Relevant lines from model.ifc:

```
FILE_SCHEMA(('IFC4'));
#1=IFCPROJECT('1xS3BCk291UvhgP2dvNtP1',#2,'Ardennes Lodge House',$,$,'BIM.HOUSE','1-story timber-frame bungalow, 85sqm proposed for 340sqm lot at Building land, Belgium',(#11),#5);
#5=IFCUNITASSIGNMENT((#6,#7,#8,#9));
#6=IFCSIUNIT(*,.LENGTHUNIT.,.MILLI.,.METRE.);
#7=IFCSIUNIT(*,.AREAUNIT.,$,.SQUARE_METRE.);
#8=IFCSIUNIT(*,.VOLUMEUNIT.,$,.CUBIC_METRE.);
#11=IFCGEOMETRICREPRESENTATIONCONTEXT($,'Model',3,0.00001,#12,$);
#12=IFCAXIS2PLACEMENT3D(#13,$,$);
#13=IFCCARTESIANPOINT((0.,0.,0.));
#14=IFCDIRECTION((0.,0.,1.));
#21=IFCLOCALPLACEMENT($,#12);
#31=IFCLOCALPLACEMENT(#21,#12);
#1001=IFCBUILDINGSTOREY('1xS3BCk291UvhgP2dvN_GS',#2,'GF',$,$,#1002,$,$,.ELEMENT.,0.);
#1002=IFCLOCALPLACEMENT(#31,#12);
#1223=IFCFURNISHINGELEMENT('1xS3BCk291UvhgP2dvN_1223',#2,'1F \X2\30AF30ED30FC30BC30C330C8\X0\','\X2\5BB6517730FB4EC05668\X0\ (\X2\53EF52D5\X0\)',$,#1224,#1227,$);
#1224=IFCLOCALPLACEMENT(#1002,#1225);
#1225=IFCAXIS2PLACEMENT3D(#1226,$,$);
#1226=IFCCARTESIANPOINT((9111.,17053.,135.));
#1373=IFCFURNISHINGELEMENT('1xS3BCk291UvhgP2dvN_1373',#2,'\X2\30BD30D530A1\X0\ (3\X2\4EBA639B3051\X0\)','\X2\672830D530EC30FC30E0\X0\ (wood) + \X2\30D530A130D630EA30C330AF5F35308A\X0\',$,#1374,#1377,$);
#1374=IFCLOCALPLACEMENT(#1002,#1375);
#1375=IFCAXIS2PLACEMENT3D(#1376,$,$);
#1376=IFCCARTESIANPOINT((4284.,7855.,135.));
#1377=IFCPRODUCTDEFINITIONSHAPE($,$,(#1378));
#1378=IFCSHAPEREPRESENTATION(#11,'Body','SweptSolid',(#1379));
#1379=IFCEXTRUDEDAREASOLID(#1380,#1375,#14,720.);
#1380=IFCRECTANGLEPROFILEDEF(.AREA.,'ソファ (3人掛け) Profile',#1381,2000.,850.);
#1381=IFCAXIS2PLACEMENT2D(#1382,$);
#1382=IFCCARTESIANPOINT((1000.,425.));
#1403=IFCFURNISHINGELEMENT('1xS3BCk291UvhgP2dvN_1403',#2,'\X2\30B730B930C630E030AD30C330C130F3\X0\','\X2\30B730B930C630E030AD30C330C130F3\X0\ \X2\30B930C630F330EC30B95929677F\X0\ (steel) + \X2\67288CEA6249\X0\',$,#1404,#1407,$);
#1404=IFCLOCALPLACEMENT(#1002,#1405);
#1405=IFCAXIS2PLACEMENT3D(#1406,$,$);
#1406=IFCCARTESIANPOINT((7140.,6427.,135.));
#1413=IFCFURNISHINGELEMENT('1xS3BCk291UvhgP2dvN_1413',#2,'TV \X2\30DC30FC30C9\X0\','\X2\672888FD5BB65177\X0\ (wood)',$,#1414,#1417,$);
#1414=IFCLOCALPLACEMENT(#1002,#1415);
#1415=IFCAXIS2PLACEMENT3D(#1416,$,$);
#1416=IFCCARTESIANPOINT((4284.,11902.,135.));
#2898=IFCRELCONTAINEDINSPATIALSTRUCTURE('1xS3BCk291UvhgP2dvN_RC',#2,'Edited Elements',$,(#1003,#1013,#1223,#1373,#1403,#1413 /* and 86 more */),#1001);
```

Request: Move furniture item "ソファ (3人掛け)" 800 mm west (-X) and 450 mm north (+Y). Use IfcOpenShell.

```python
import ifcopenshell
import ifcopenshell.api.geometry
import ifcopenshell.util.placement

model = ifcopenshell.open("model.ifc")

item = model.by_guid("1xS3BCk291UvhgP2dvN_1373")
matrix = ifcopenshell.util.placement.get_local_placement(item.ObjectPlacement)
matrix[0, 3] -= 800.0
matrix[1, 3] += 450.0
ifcopenshell.api.geometry.edit_object_placement(model, product=item, matrix=matrix, is_si=False)

print(ifcopenshell.util.placement.get_local_placement(item.ObjectPlacement).round(3) + 0.0)

model.write("model_updated.ifc")
```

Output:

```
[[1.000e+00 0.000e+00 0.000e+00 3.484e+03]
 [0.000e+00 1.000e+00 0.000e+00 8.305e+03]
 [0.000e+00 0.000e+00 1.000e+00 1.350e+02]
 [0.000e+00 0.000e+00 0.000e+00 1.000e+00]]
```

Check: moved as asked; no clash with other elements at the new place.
